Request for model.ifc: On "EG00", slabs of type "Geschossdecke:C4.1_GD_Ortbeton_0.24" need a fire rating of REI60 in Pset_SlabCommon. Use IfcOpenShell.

First a look at what the model holds.

```python
import ifcopenshell
import ifcopenshell.util.element

model = ifcopenshell.open("model.ifc")
print(model.schema)
storey = next(s for s in model.by_type("IfcBuildingStorey") if s.Name == "EG00")
slabs = [e for e in ifcopenshell.util.element.get_decomposition(storey) if e.is_a("IfcSlab")]
seen = {}
for e in slabs:
    element_type = ifcopenshell.util.element.get_type(e)
    key = (element_type.Name if element_type != e and element_type else None, ifcopenshell.util.element.get_pset(e, "Pset_SlabCommon", "FireRating"))
    seen[key] = seen.get(key, 0) + 1
for (name, value), count in sorted(seen.items(), key=str):
    print(count, "x", name, "|", value)
```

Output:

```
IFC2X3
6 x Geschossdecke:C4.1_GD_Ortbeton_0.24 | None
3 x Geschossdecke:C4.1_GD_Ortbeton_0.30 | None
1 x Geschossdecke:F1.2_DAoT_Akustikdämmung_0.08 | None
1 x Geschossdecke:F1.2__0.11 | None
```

```python
import ifcopenshell
import ifcopenshell.api.pset
import ifcopenshell.util.element

model = ifcopenshell.open("model.ifc")

storey = next(s for s in model.by_type("IfcBuildingStorey") if s.Name == "EG00")
slabs = [e for e in ifcopenshell.util.element.get_decomposition(storey) if e.is_a("IfcSlab")]

count = 0
for e in slabs:
    element_type = ifcopenshell.util.element.get_type(e)
    if element_type in (None, e) or element_type.Name != "Geschossdecke:C4.1_GD_Ortbeton_0.24":
        continue
    # add_pset returns the element's existing set when there is one.
    pset = ifcopenshell.api.pset.add_pset(model, product=e, name="Pset_SlabCommon")
    ifcopenshell.api.pset.edit_pset(model, pset=pset, properties={"FireRating": "REI60"})
    count += 1

print(count, "slabs updated")

model.write("model_updated.ifc")
```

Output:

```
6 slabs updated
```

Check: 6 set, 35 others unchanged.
